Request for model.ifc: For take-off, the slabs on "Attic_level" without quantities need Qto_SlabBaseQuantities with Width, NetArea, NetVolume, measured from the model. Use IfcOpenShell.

First a look at what the model holds.

```python
import ifcopenshell
import ifcopenshell.util.element
import ifcopenshell.util.unit

model = ifcopenshell.open("model.ifc")
print(model.schema)
for unit_type in ("LENGTHUNIT", "AREAUNIT", "VOLUMEUNIT"):
    print(unit_type, ifcopenshell.util.unit.calculate_unit_scale(model, unit_type))
storey = next(s for s in model.by_type("IfcBuildingStorey") if s.Name == "Attic_level")
slabs = [e for e in ifcopenshell.util.element.get_decomposition(storey) if e.is_a("IfcSlab")]
for e in sorted(slabs, key=lambda e: e.id()):
    print(e.id(), e.is_a(), e.Name, list(ifcopenshell.util.element.get_psets(e, qtos_only=True)), sep=" | ")
```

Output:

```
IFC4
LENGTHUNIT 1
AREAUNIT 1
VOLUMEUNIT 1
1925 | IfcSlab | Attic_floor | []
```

```python
import ifcopenshell
import ifcopenshell.api.pset
import ifcopenshell.geom
import ifcopenshell.util.element
import ifcopenshell.util.shape
import ifcopenshell.util.unit

model = ifcopenshell.open("model.ifc")
unit_scale = ifcopenshell.util.unit.calculate_unit_scale(model)
area_scale = ifcopenshell.util.unit.calculate_unit_scale(model, "AREAUNIT")
volume_scale = ifcopenshell.util.unit.calculate_unit_scale(model, "VOLUMEUNIT")
settings = ifcopenshell.geom.settings()

storey = next(s for s in model.by_type("IfcBuildingStorey") if s.Name == "Attic_level")
slabs = [e for e in ifcopenshell.util.element.get_decomposition(storey) if e.is_a("IfcSlab")]

for e in sorted(slabs, key=lambda e: e.id()):
    if ifcopenshell.util.element.get_psets(e, qtos_only=True, should_inherit=False):
        continue
    # Geometry comes back in metres, in the element's own axes.
    shape = ifcopenshell.geom.create_shape(settings, e)
    values = {
        "Width": ifcopenshell.util.shape.get_z(shape.geometry) / unit_scale,
        "NetArea": ifcopenshell.util.shape.get_footprint_area(shape.geometry) / area_scale,
        "NetVolume": ifcopenshell.util.shape.get_volume(shape.geometry) / volume_scale,
    }
    qto = ifcopenshell.api.pset.add_qto(model, product=e, name="Qto_SlabBaseQuantities")
    ifcopenshell.api.pset.edit_qto(model, qto=qto, properties=values)
    print(e.id(), {k: round(v, 3) for k, v in values.items()})

model.write("model_edited.ifc")
```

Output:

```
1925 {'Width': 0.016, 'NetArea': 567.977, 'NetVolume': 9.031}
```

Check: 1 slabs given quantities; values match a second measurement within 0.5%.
